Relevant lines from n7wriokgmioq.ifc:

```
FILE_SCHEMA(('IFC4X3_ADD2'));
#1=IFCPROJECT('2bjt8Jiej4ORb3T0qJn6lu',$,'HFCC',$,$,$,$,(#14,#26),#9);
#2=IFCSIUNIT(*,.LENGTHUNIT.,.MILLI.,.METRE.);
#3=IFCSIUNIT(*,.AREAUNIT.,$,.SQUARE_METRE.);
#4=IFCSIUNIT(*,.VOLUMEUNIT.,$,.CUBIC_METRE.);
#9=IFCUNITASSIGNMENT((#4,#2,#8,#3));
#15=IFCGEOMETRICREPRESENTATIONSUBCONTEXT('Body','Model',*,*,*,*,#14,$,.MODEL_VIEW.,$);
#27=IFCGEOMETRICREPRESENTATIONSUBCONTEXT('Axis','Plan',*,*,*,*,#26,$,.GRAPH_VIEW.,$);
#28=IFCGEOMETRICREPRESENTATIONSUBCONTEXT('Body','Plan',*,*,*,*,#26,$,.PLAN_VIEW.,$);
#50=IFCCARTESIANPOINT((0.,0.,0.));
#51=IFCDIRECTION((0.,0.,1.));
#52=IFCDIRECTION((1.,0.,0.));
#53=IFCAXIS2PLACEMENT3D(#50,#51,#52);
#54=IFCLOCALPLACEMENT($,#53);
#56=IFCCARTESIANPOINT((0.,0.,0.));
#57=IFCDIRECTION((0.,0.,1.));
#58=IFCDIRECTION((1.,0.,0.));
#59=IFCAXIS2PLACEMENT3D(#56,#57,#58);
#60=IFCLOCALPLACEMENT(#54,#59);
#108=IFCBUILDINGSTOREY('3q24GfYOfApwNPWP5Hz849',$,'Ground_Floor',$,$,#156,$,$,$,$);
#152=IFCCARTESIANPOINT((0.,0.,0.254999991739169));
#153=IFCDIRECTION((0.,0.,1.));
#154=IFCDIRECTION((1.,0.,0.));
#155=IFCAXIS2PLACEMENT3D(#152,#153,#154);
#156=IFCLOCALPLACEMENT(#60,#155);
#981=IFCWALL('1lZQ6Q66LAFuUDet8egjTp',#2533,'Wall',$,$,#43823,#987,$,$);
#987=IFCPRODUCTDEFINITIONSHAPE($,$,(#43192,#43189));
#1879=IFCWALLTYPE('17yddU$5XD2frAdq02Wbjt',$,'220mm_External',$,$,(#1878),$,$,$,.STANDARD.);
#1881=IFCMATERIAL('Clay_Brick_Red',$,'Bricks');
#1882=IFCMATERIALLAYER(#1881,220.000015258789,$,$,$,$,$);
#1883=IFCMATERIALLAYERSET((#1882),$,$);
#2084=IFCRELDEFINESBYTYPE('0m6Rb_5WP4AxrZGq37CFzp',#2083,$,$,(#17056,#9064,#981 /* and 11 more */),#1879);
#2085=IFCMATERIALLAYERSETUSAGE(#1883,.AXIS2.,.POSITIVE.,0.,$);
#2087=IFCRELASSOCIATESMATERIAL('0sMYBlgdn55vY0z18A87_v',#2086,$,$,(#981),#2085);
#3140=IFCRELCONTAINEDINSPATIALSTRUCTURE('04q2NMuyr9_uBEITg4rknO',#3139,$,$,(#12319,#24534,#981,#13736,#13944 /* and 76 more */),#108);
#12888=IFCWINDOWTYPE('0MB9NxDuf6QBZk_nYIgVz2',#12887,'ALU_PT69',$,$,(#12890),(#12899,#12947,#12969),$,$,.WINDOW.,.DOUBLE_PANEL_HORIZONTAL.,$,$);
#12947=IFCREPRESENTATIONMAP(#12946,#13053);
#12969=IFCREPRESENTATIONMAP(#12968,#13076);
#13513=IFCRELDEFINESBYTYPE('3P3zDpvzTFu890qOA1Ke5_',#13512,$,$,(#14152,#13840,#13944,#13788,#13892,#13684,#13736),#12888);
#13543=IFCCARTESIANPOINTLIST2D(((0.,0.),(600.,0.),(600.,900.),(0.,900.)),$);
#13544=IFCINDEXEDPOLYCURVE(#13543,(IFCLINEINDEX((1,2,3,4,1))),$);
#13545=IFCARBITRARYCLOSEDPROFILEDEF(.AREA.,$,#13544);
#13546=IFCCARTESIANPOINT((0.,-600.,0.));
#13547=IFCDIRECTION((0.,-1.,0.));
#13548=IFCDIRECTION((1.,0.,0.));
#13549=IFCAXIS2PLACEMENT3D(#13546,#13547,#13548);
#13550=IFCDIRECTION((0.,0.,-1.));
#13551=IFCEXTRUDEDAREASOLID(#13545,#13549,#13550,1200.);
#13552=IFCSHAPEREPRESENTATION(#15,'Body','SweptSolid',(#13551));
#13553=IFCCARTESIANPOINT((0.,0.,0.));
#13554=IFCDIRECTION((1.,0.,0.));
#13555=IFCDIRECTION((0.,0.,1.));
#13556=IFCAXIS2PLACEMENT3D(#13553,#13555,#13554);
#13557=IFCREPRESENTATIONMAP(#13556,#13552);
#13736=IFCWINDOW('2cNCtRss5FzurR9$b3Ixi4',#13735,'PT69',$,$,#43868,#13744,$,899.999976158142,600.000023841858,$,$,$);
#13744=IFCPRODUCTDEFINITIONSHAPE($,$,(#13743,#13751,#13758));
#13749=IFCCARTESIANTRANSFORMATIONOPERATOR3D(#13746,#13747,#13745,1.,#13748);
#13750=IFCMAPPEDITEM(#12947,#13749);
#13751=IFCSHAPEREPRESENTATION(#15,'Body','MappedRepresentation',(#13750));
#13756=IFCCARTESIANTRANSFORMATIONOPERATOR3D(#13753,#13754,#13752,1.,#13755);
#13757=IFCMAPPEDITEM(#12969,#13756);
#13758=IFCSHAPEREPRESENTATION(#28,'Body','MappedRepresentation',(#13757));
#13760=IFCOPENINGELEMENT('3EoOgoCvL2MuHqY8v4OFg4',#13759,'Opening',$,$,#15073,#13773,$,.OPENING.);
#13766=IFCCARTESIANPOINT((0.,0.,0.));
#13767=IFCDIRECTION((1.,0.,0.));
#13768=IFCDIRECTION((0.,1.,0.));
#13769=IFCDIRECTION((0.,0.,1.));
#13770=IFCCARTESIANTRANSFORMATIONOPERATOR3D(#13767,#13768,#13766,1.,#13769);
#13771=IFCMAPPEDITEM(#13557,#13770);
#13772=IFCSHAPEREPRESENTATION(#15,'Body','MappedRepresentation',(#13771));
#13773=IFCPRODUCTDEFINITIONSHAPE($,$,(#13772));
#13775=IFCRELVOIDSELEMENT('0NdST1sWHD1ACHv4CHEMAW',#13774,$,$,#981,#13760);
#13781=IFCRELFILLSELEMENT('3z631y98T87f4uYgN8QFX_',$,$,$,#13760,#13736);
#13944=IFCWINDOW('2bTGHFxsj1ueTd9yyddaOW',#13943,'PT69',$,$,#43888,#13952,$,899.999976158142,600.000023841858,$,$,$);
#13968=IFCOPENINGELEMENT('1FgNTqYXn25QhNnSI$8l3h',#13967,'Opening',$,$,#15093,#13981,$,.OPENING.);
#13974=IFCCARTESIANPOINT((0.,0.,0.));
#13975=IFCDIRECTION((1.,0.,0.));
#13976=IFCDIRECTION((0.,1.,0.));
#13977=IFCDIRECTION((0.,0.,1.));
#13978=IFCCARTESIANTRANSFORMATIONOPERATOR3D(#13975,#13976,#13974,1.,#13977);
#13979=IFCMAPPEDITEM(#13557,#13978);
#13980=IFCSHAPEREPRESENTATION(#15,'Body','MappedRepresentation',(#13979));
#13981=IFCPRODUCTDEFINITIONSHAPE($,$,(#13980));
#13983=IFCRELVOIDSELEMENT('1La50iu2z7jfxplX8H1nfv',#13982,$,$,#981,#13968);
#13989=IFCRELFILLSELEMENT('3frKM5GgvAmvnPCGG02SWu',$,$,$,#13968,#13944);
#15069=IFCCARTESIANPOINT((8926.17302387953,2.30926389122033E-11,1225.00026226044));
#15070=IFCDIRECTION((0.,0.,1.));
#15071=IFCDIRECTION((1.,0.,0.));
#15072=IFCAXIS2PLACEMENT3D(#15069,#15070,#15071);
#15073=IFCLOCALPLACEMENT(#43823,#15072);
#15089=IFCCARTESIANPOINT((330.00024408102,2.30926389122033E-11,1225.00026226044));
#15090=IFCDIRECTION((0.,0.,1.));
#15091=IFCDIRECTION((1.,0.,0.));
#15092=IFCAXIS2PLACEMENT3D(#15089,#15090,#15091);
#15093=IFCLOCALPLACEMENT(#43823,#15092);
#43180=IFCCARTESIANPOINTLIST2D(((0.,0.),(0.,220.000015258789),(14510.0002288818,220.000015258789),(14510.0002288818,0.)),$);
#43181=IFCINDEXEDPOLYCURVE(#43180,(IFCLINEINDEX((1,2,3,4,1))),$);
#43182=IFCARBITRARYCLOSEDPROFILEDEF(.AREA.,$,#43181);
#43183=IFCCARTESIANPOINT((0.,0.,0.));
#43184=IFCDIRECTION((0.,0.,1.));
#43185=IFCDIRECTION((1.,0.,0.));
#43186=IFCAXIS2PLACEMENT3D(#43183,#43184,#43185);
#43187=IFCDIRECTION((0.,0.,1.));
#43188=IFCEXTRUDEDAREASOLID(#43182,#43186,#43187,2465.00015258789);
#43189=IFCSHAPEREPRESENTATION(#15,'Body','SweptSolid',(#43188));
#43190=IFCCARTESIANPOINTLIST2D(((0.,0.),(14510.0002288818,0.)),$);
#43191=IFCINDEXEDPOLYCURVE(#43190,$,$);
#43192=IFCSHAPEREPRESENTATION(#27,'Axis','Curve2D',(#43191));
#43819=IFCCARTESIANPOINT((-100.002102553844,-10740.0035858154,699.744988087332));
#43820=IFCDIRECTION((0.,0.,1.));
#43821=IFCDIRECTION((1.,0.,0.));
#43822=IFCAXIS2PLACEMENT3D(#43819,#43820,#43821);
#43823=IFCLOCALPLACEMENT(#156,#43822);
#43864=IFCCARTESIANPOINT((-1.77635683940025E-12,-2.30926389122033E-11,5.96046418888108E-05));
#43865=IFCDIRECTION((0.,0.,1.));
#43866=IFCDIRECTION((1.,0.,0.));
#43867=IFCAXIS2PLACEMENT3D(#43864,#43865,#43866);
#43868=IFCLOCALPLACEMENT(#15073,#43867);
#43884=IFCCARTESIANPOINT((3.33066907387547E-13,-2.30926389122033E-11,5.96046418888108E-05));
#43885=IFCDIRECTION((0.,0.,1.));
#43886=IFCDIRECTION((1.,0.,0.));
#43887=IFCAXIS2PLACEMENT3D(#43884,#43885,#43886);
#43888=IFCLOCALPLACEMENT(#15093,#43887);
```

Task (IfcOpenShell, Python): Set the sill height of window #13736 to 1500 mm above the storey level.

```python
import numpy as np
import ifcopenshell
import ifcopenshell.api.geometry
import ifcopenshell.geom
import ifcopenshell.util.element
import ifcopenshell.util.placement
import ifcopenshell.util.shape
import ifcopenshell.util.unit

model = ifcopenshell.open("n7wriokgmioq.ifc")
unit_scale = ifcopenshell.util.unit.calculate_unit_scale(model)

window = model.by_id(13736)
opening = window.FillsVoids[0].RelatingOpeningElement
storey = ifcopenshell.util.element.get_container(window, ifc_class="IfcBuildingStorey")
level = ifcopenshell.util.placement.get_local_placement(storey.ObjectPlacement)[2, 3]

# The opening's origin need not be at the sill, so measure its lowest point.
shape = ifcopenshell.geom.create_shape(ifcopenshell.geom.settings(), opening)
bottom = ifcopenshell.util.shape.get_shape_bottom_elevation(shape, shape.geometry) / unit_scale
dz = level + 1500.0 - bottom

shift = np.array([0.0, 0.0, dz])
# The window is placed relative to its opening, so it follows when the opening moves.
matrix = ifcopenshell.util.placement.get_local_placement(opening.ObjectPlacement)
matrix[:3, 3] += shift
ifcopenshell.api.geometry.edit_object_placement(
    model, product=opening, matrix=matrix, is_si=False, should_transform_children=True
)

print(f"moved by {dz * unit_scale:+.3f} m")

model.write("n7wriokgmioq_edited.ifc")
```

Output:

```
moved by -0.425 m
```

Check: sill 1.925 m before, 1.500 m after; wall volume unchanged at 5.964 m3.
